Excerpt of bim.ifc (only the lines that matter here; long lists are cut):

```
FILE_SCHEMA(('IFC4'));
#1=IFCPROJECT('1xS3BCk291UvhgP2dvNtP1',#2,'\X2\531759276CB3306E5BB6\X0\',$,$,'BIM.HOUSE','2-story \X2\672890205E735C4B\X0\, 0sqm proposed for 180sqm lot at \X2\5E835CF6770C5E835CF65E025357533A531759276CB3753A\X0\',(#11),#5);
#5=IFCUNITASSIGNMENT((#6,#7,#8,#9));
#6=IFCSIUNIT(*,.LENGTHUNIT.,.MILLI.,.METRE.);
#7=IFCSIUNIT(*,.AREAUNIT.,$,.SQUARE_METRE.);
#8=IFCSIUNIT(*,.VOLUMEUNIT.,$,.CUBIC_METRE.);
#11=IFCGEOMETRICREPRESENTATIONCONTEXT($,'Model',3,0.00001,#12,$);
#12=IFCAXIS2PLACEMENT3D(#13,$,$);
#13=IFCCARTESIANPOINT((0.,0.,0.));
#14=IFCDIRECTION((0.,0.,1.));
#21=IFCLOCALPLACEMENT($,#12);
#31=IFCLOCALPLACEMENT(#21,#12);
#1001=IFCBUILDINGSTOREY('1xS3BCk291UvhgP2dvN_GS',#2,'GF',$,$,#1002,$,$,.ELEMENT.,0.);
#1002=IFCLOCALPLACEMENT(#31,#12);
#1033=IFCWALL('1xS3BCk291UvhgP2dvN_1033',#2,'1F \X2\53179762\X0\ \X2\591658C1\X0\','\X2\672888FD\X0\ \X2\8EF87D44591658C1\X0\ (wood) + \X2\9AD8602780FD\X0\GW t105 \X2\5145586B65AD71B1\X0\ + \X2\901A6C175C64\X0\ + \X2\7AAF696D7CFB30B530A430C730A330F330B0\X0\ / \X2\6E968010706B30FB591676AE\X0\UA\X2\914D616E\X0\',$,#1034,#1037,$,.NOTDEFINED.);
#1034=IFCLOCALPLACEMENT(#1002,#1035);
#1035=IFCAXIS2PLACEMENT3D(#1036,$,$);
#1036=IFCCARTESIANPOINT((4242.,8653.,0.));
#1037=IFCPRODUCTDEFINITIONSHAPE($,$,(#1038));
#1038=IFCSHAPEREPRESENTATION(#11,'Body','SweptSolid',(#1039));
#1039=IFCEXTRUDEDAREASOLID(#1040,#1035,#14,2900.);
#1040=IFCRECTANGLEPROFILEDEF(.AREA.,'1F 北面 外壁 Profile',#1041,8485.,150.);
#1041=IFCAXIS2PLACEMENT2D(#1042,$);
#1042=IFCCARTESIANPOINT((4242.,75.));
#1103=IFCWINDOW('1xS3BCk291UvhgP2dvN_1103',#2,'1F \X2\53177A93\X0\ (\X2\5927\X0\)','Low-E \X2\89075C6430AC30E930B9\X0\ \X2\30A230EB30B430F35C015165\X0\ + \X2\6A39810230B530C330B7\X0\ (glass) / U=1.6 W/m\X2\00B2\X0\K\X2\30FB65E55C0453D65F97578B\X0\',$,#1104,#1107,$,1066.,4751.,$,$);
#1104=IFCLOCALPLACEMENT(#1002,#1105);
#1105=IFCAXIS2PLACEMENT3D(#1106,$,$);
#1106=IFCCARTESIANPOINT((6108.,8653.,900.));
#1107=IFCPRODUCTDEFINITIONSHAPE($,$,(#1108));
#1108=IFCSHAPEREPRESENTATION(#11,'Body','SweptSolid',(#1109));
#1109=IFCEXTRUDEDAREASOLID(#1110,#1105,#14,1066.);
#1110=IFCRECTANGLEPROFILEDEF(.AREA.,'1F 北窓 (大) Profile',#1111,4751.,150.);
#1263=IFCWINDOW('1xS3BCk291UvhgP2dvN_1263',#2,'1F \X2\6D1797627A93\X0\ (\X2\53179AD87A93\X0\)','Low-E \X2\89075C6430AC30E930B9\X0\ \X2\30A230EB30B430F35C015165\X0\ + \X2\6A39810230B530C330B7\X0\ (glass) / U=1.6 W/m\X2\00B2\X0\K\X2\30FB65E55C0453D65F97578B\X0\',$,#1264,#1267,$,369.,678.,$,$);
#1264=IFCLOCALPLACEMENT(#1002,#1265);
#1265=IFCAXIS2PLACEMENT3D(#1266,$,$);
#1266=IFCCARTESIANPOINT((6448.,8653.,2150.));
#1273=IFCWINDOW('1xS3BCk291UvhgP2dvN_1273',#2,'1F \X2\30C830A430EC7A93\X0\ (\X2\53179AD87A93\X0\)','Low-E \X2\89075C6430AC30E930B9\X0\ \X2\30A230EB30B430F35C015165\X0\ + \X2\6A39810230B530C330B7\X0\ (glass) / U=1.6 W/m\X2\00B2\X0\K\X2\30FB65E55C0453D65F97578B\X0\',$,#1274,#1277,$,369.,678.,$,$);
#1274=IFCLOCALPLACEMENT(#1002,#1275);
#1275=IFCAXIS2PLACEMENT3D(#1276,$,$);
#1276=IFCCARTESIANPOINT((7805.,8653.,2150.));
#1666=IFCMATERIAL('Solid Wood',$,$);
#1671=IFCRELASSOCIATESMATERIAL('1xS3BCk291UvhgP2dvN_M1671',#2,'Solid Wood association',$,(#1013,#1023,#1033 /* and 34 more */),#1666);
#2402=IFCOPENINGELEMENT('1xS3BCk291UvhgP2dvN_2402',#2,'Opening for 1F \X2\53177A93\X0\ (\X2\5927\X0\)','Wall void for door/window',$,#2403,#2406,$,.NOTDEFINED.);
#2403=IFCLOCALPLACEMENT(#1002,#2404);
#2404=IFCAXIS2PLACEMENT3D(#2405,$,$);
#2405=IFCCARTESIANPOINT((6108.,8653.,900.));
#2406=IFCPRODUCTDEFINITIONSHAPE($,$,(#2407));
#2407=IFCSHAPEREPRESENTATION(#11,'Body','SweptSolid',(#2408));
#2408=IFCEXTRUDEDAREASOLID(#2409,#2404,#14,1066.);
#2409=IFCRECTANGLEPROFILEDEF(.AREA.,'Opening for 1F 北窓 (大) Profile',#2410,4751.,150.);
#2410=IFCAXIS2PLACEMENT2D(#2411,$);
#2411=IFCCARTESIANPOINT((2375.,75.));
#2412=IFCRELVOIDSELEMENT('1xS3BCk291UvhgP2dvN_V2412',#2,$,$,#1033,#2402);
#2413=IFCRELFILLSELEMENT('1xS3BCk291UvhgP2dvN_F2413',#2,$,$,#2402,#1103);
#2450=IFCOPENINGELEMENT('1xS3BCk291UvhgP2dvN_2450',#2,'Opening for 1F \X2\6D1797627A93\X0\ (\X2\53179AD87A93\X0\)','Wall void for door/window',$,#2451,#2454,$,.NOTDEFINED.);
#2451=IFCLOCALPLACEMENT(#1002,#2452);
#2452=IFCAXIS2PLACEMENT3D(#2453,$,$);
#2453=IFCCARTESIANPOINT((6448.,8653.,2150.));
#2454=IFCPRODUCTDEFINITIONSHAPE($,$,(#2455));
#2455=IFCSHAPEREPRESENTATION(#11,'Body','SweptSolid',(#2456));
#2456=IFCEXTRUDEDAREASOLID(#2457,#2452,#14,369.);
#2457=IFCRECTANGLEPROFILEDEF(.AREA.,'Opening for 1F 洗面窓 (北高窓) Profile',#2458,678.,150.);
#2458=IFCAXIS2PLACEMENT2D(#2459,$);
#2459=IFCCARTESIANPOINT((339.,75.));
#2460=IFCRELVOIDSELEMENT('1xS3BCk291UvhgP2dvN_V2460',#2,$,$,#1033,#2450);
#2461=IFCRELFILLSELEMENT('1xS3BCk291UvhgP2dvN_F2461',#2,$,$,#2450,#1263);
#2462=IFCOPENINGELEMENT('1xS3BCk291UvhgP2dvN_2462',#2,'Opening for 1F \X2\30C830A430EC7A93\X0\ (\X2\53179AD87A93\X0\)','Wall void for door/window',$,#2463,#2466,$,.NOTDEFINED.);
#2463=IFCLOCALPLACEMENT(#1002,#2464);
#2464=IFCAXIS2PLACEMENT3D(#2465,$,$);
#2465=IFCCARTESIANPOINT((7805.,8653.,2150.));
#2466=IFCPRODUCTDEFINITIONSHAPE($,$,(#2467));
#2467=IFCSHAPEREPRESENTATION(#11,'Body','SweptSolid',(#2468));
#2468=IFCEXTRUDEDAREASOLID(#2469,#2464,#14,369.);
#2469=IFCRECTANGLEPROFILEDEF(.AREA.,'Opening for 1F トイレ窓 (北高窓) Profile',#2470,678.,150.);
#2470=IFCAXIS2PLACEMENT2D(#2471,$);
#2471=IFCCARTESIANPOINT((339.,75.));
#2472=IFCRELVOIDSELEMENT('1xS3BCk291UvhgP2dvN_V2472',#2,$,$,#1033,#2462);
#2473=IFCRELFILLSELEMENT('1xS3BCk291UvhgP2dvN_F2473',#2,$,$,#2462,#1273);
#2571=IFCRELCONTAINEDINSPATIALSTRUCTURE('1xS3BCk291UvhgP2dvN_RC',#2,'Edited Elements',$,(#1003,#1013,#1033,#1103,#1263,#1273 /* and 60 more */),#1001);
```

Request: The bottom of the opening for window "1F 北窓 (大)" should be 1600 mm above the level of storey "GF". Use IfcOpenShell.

```python
import numpy as np
import ifcopenshell
import ifcopenshell.api.geometry
import ifcopenshell.geom
import ifcopenshell.util.element
import ifcopenshell.util.placement
import ifcopenshell.util.shape
import ifcopenshell.util.unit

model = ifcopenshell.open("bim.ifc")
unit_scale = ifcopenshell.util.unit.calculate_unit_scale(model)

window = model.by_guid("1xS3BCk291UvhgP2dvN_1103")
opening = window.FillsVoids[0].RelatingOpeningElement
storey = ifcopenshell.util.element.get_container(window, ifc_class="IfcBuildingStorey")
level = ifcopenshell.util.placement.get_local_placement(storey.ObjectPlacement)[2, 3]

# The opening's origin need not be at the sill, so measure its lowest point.
shape = ifcopenshell.geom.create_shape(ifcopenshell.geom.settings(), opening)
bottom = ifcopenshell.util.shape.get_shape_bottom_elevation(shape, shape.geometry) / unit_scale
dz = level + 1600.0 - bottom

shift = np.array([0.0, 0.0, dz])
# The window is not placed relative to its opening, so move both.
for product in (opening, window):
    matrix = ifcopenshell.util.placement.get_local_placement(product.ObjectPlacement)
    matrix[:3, 3] += shift
    ifcopenshell.api.geometry.edit_object_placement(model, product=product, matrix=matrix, is_si=False)

print(f"moved by {dz * unit_scale:+.3f} m")

model.write("bim-out.ifc")
```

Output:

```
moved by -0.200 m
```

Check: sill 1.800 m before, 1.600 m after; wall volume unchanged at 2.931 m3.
